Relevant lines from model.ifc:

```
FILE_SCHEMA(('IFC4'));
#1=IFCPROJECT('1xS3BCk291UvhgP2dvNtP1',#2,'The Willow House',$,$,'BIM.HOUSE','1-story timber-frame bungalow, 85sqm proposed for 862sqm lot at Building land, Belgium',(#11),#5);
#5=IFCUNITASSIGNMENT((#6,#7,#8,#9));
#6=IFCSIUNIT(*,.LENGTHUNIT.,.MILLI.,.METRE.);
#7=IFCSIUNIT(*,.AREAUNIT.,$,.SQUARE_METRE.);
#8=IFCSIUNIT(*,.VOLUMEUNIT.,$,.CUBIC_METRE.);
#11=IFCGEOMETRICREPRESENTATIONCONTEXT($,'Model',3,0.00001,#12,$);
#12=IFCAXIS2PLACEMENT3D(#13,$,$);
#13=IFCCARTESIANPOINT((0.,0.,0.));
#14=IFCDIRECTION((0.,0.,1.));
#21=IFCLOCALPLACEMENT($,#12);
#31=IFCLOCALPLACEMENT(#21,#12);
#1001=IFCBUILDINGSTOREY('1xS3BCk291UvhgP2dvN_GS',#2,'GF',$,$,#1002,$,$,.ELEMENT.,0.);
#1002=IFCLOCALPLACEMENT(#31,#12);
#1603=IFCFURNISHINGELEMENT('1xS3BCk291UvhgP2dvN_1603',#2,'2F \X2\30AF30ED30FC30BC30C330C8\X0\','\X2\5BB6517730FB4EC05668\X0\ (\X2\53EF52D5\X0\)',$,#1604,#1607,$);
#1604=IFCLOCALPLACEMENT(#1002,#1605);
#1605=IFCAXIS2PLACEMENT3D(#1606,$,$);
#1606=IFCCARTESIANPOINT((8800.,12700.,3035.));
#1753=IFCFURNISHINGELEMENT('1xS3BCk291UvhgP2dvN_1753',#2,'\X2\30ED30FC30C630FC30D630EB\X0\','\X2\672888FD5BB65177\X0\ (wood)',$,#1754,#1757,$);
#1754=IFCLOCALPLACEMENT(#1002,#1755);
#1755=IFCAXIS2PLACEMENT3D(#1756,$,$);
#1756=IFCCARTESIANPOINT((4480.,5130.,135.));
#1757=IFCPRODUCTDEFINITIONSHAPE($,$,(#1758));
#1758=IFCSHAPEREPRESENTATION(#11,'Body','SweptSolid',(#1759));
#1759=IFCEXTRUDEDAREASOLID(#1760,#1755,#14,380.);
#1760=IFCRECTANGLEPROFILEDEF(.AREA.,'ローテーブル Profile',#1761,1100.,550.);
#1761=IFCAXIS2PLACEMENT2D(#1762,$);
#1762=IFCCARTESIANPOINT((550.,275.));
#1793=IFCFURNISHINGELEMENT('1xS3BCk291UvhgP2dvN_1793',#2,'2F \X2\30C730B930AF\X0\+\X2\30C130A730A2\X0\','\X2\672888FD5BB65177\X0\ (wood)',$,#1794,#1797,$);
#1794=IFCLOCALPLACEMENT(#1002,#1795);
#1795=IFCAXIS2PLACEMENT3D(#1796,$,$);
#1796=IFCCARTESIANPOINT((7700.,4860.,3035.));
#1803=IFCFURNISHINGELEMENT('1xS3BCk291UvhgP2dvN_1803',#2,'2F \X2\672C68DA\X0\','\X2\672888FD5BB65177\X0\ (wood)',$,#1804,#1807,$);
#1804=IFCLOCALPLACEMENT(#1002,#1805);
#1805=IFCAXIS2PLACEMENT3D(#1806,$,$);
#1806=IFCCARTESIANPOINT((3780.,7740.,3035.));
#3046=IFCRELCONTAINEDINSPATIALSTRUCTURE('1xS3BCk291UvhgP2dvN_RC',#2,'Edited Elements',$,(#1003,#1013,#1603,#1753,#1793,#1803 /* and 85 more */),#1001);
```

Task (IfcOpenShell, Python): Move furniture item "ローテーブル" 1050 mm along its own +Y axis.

```python
import ifcopenshell
import ifcopenshell.api.geometry
import ifcopenshell.util.placement

model = ifcopenshell.open("model.ifc")

item = model.by_id(1753)
matrix = ifcopenshell.util.placement.get_local_placement(item.ObjectPlacement)
matrix[:3, 3] += matrix[:3, 1] * 1050.0
ifcopenshell.api.geometry.edit_object_placement(model, product=item, matrix=matrix, is_si=False)

print(ifcopenshell.util.placement.get_local_placement(item.ObjectPlacement).round(3) + 0.0)

model.write("model_rev.ifc")
```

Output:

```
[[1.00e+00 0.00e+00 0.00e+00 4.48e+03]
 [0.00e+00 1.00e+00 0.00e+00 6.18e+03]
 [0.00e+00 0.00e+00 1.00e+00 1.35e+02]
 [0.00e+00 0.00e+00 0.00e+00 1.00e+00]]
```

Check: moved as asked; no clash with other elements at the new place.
